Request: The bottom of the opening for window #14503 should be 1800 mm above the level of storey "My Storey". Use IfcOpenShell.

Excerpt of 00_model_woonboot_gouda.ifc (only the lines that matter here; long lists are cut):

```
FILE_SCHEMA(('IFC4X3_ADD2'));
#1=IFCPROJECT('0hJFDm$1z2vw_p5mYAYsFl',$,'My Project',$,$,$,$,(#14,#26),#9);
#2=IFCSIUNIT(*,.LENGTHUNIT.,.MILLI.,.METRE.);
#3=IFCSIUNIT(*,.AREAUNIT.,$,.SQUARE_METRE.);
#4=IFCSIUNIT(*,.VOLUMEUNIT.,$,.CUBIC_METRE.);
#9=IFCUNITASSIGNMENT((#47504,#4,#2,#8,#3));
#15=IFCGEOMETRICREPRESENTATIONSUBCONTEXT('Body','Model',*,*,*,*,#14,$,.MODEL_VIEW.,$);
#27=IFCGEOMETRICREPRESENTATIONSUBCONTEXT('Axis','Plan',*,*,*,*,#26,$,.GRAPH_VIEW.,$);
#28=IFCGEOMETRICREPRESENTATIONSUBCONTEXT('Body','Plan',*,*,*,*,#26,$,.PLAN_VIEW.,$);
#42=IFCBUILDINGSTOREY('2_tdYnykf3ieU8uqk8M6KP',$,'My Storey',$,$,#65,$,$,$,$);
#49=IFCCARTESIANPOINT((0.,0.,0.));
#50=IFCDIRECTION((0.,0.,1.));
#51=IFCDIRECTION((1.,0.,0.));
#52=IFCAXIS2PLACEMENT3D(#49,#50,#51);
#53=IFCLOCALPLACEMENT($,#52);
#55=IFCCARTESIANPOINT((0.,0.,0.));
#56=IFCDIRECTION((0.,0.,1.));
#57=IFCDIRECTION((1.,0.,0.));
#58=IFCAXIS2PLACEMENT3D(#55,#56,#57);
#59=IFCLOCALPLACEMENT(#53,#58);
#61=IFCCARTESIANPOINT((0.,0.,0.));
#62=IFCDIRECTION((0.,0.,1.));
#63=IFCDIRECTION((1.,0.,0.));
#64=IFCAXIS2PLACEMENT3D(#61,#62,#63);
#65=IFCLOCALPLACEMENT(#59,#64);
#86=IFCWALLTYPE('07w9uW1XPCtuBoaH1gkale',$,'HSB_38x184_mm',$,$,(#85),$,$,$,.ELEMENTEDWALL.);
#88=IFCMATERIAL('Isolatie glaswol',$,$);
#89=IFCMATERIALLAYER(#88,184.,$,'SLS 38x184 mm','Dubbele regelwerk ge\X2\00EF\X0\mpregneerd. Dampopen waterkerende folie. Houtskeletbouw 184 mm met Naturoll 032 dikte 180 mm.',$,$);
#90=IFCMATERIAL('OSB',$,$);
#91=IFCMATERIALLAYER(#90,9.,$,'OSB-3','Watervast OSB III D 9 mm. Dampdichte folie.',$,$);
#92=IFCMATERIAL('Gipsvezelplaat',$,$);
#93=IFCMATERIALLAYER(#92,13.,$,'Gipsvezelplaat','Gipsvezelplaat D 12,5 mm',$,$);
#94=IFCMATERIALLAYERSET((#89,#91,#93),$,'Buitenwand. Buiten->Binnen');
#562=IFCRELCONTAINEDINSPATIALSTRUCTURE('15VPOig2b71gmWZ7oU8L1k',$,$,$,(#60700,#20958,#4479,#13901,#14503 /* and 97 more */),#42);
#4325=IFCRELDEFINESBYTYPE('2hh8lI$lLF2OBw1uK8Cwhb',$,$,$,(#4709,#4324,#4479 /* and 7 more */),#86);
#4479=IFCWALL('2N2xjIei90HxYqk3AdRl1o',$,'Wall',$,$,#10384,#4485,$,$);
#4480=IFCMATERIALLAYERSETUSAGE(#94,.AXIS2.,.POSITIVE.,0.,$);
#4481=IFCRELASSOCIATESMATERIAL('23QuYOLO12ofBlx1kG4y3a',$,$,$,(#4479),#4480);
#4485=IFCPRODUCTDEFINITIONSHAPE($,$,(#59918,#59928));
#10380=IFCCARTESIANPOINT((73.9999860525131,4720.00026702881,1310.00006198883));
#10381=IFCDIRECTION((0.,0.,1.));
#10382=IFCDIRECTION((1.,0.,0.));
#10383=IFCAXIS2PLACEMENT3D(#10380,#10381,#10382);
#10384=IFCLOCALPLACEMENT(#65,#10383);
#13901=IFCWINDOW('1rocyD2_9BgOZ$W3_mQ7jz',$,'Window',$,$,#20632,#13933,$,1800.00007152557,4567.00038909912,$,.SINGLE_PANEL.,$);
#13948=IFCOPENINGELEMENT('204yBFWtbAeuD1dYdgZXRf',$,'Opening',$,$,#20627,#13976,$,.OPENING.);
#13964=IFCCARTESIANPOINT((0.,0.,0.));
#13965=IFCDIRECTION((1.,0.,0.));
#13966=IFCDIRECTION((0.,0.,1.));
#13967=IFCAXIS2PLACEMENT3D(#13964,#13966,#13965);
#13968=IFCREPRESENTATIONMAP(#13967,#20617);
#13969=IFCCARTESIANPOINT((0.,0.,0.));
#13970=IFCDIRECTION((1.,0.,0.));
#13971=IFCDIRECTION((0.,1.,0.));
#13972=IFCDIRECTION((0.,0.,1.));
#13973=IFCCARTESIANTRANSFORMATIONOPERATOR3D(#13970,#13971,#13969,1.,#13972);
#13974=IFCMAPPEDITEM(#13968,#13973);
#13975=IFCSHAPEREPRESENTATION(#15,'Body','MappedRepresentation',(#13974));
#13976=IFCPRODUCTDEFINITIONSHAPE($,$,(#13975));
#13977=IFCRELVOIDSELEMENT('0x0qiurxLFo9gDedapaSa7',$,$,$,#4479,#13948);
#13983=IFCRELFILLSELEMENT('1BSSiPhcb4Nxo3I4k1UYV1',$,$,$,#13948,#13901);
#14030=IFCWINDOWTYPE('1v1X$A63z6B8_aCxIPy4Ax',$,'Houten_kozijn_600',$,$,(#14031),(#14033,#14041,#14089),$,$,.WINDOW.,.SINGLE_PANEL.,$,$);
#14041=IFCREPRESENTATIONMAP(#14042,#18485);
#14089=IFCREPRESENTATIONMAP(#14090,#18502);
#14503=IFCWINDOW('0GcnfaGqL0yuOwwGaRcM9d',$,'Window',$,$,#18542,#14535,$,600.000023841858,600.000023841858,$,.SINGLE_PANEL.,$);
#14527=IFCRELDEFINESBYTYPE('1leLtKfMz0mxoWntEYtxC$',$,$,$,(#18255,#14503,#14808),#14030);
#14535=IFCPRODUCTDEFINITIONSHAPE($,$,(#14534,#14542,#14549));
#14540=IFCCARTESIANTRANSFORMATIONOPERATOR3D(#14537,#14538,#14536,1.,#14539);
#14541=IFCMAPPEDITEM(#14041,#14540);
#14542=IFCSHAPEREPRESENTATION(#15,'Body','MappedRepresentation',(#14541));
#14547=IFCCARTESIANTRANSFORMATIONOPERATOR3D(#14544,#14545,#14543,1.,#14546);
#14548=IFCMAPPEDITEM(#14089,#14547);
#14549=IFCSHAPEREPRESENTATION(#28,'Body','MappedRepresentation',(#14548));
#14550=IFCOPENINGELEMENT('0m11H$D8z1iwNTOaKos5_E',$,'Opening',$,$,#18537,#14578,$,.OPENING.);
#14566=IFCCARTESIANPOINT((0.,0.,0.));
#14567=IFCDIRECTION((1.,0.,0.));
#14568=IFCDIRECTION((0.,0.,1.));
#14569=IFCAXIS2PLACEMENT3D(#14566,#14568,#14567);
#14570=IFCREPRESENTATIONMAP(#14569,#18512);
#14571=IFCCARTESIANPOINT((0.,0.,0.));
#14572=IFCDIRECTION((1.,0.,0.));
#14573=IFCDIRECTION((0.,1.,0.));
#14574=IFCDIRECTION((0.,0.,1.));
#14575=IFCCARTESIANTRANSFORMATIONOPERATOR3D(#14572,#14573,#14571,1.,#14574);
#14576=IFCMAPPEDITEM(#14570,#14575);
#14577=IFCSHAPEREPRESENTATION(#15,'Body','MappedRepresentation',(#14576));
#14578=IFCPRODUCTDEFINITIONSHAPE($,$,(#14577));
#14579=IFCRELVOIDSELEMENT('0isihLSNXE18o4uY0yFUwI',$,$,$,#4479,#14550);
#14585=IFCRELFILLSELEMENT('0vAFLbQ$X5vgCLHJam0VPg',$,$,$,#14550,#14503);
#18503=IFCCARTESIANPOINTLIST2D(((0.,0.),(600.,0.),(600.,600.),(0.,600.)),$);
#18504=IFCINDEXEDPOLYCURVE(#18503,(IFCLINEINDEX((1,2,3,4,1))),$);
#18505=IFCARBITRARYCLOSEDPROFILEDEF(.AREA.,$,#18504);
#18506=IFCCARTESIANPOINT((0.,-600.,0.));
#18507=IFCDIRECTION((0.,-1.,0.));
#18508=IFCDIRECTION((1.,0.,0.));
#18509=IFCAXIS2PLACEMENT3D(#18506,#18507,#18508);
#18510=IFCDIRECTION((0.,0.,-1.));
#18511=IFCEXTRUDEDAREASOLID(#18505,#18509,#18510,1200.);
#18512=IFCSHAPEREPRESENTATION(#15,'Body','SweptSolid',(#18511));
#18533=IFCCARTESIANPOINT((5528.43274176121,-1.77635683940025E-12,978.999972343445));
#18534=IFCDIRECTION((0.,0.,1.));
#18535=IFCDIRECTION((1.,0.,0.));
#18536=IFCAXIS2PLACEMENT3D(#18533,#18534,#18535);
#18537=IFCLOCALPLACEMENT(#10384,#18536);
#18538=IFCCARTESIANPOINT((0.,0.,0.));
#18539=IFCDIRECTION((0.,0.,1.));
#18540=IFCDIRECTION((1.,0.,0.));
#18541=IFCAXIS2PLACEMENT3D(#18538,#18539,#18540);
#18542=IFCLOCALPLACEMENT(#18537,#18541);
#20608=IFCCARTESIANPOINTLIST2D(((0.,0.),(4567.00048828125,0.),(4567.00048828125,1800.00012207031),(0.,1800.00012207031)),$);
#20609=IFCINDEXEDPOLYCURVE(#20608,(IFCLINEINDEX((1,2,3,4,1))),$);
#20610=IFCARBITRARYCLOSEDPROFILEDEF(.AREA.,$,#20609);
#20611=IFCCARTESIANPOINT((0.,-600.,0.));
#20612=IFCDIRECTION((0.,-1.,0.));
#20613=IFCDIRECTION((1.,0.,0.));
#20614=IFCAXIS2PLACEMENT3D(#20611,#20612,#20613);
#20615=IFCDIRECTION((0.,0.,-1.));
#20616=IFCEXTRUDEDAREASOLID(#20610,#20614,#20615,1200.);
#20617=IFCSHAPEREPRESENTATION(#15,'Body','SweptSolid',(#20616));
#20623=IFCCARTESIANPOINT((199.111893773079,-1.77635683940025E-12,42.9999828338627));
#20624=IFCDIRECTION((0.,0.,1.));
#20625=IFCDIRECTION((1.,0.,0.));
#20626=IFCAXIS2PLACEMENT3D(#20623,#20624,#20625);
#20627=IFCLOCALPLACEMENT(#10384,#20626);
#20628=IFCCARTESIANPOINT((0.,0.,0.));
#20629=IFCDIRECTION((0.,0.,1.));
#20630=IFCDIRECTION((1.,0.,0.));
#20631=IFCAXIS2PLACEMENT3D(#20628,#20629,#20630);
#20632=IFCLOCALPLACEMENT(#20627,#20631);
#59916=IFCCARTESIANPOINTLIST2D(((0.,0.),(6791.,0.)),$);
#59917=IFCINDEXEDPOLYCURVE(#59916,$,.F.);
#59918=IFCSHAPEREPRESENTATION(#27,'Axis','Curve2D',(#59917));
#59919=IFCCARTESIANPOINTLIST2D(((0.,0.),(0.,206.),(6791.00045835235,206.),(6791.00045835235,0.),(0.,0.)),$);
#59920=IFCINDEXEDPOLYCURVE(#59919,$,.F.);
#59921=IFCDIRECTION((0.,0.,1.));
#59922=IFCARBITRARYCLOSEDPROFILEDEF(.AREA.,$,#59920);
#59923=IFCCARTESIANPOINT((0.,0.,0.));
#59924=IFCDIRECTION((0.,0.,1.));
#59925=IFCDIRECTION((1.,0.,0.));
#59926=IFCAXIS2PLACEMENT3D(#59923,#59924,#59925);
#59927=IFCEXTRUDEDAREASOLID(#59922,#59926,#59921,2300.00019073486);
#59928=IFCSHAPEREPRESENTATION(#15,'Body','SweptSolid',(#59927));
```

```python
import numpy as np
import ifcopenshell
import ifcopenshell.api.geometry
import ifcopenshell.geom
import ifcopenshell.util.element
import ifcopenshell.util.placement
import ifcopenshell.util.shape
import ifcopenshell.util.unit

model = ifcopenshell.open("00_model_woonboot_gouda.ifc")
unit_scale = ifcopenshell.util.unit.calculate_unit_scale(model)

window = model.by_guid("0GcnfaGqL0yuOwwGaRcM9d")
opening = window.FillsVoids[0].RelatingOpeningElement
storey = ifcopenshell.util.element.get_container(window, ifc_class="IfcBuildingStorey")
level = ifcopenshell.util.placement.get_local_placement(storey.ObjectPlacement)[2, 3]

# The opening's origin need not be at the sill, so measure its lowest point.
shape = ifcopenshell.geom.create_shape(ifcopenshell.geom.settings(), opening)
bottom = ifcopenshell.util.shape.get_shape_bottom_elevation(shape, shape.geometry) / unit_scale
dz = level + 1.8 / unit_scale - bottom

shift = np.array([0.0, 0.0, dz])
# The window is placed relative to its opening, so it follows when the opening moves.
matrix = ifcopenshell.util.placement.get_local_placement(opening.ObjectPlacement)
matrix[:3, 3] += shift
ifcopenshell.api.geometry.edit_object_placement(
    model, product=opening, matrix=matrix, is_si=False, should_transform_children=True
)

print(f"moved by {dz * unit_scale:+.3f} m")

model.write("00_model_woonboot_gouda_edited.ifc")
```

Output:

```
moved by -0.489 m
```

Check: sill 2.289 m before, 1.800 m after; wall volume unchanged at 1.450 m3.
